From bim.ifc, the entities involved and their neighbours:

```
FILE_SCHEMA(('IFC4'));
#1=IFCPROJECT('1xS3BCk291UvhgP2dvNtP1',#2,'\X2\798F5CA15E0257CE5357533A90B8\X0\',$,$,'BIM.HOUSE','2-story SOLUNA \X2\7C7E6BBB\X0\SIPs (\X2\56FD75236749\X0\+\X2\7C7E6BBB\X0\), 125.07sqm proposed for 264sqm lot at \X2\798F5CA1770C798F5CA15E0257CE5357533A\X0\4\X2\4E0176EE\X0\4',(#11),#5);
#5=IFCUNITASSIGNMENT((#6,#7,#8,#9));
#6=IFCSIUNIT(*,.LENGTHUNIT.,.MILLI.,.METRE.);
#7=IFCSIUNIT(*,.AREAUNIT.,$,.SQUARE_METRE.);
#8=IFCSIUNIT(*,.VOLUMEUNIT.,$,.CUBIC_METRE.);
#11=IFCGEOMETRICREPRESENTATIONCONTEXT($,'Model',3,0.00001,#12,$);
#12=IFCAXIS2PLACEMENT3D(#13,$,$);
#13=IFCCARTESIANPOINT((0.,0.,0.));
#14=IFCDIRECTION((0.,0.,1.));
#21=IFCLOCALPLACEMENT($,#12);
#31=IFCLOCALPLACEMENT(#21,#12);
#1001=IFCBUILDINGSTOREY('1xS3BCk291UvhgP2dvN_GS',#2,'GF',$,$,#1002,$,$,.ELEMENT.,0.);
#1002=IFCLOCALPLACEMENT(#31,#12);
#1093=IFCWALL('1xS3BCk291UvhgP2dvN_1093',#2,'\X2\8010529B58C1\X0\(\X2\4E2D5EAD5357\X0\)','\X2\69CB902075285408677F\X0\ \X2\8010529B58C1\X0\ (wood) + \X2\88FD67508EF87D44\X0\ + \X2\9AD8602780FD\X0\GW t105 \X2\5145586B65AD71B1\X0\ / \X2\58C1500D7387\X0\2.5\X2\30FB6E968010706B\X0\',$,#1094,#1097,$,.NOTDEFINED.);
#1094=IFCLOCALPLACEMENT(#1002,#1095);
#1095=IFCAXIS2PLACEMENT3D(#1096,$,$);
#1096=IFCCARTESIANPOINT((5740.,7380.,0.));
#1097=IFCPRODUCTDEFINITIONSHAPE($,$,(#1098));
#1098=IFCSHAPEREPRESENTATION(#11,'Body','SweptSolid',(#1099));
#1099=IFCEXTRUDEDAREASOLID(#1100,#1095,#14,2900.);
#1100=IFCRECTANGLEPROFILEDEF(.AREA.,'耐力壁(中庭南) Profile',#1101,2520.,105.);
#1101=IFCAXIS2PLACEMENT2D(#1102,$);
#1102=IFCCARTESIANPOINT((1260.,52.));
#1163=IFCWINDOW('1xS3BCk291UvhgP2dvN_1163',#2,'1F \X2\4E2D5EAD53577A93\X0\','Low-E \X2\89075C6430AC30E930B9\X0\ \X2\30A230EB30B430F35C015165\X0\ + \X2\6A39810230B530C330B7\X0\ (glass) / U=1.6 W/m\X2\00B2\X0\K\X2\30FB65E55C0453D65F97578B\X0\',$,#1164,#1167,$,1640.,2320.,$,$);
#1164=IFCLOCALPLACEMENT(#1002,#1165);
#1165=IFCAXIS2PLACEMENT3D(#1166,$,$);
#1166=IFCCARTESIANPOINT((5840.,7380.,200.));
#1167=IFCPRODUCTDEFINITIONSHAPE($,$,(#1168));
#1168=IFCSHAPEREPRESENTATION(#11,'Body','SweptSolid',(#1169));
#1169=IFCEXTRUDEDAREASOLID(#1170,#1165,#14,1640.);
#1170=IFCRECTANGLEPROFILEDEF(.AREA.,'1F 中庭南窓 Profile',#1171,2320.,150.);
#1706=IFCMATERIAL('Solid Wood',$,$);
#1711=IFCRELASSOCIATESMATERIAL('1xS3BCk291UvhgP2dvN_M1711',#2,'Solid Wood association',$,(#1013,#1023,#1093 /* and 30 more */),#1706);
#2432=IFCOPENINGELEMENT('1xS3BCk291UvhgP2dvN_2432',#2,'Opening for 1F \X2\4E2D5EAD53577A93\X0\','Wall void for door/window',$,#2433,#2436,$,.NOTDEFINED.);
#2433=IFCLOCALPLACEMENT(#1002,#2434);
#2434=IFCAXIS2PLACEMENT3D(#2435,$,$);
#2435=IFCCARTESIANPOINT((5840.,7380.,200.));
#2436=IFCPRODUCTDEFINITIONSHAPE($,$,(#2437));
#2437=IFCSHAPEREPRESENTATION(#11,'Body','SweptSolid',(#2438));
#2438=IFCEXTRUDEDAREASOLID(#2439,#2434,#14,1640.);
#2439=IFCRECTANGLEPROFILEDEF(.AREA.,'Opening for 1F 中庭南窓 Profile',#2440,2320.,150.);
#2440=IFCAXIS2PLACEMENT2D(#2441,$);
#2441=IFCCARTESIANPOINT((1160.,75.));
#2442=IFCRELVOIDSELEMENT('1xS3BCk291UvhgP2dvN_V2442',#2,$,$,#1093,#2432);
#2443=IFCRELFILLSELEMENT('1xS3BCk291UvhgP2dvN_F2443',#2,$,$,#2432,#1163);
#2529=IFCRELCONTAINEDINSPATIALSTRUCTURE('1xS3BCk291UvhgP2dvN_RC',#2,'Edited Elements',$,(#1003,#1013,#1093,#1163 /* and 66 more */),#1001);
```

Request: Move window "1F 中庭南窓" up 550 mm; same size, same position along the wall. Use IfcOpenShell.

```python
import numpy as np
import ifcopenshell
import ifcopenshell.api.geometry
import ifcopenshell.util.placement
import ifcopenshell.util.unit

model = ifcopenshell.open("bim.ifc")
unit_scale = ifcopenshell.util.unit.calculate_unit_scale(model)

window = model.by_guid("1xS3BCk291UvhgP2dvN_1163")
opening = window.FillsVoids[0].RelatingOpeningElement
dz = 0.55 / unit_scale

shift = np.array([0.0, 0.0, dz])
# The window is not placed relative to its opening, so move both.
for product in (opening, window):
    matrix = ifcopenshell.util.placement.get_local_placement(product.ObjectPlacement)
    matrix[:3, 3] += shift
    ifcopenshell.api.geometry.edit_object_placement(model, product=product, matrix=matrix, is_si=False)

print(f"moved by {dz * unit_scale:+.3f} m")

model.write("bim-out.ifc")
```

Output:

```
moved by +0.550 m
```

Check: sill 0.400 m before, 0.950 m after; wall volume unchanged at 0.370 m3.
